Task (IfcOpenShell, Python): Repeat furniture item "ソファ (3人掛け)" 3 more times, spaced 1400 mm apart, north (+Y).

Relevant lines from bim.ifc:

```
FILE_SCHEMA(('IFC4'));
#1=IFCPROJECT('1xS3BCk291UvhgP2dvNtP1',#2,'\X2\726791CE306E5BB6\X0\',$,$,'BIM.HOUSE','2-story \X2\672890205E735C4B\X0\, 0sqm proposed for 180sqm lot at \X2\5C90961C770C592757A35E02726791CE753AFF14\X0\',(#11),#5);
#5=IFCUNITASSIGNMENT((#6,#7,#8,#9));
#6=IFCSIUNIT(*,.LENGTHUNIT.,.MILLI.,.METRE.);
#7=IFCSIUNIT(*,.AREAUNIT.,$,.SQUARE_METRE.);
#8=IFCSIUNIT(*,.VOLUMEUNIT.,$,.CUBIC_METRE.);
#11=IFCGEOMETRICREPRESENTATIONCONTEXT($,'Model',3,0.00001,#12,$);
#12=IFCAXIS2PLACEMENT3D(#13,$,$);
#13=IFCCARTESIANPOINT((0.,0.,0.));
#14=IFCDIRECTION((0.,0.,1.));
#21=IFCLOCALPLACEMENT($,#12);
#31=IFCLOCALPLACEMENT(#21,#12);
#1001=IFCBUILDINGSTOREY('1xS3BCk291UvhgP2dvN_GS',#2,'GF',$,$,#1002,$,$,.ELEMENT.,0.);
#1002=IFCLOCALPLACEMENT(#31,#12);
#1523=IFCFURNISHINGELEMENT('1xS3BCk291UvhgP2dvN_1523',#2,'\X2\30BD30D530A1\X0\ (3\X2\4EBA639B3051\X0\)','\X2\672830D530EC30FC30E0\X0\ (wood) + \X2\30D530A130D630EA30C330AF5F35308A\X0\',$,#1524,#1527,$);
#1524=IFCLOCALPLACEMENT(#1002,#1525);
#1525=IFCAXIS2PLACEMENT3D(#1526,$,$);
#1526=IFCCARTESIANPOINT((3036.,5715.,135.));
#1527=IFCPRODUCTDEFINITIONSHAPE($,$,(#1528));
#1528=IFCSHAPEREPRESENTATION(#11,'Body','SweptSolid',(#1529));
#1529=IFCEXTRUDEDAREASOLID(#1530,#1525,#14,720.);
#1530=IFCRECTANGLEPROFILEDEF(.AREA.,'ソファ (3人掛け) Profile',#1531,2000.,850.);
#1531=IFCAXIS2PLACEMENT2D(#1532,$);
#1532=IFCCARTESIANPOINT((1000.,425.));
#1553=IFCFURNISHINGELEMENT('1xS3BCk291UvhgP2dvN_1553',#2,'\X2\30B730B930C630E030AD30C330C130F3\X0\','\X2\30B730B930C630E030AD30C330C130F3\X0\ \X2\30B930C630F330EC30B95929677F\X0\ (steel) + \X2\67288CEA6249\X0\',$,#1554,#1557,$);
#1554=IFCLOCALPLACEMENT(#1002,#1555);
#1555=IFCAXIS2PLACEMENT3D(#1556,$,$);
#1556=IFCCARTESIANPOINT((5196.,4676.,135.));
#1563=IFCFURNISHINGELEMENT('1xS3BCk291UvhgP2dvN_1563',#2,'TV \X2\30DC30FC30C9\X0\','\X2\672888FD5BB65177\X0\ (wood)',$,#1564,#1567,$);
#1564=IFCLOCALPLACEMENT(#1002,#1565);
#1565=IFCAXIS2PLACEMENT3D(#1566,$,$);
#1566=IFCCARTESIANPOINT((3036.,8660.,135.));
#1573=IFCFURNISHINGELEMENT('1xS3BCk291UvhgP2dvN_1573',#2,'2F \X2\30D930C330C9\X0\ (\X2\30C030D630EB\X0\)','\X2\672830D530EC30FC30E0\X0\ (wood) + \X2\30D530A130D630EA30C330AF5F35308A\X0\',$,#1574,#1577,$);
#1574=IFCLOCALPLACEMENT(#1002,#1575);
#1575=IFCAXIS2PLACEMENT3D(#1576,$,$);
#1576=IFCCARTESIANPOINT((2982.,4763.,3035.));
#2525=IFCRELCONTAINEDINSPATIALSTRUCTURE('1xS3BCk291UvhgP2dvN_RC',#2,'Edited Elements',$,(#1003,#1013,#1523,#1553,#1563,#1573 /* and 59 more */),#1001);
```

```python
import numpy as np
import ifcopenshell
import ifcopenshell.api.geometry
import ifcopenshell.api.root
import ifcopenshell.util.element
import ifcopenshell.util.placement

model = ifcopenshell.open("bim.ifc")


def reuse_history(source, copy):
    """copy_class also copies each property set's owner history, people and application; keep the originals."""
    for rel in copy.IsDefinedBy:
        if rel.is_a("IfcRelDefinesByProperties") and (history := rel.RelatingPropertyDefinition.OwnerHistory):
            rel.RelatingPropertyDefinition.OwnerHistory = source.OwnerHistory
            ifcopenshell.util.element.remove_deep2(model, history)


source = model.by_id(1523)
base = ifcopenshell.util.placement.get_local_placement(source.ObjectPlacement)
step = np.array([0.0, 1.0, 0.0]) * 1400.0

for i in range(1, 4):
    copy = ifcopenshell.api.root.copy_class(model, product=source)
    copy.Representation = ifcopenshell.util.element.copy_deep(
        model, source.Representation, exclude=["IfcGeometricRepresentationContext", "IfcRepresentationMap"]
    )
    reuse_history(source, copy)
    matrix = base.copy()
    matrix[:3, 3] += i * step
    print("added at", matrix[:3, 3].round(3) + 0.0)
    ifcopenshell.api.geometry.edit_object_placement(model, product=copy, matrix=matrix, is_si=False)

model.write("bim-out.ifc")
```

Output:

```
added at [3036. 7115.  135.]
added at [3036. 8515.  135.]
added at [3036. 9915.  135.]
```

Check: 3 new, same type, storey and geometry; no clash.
